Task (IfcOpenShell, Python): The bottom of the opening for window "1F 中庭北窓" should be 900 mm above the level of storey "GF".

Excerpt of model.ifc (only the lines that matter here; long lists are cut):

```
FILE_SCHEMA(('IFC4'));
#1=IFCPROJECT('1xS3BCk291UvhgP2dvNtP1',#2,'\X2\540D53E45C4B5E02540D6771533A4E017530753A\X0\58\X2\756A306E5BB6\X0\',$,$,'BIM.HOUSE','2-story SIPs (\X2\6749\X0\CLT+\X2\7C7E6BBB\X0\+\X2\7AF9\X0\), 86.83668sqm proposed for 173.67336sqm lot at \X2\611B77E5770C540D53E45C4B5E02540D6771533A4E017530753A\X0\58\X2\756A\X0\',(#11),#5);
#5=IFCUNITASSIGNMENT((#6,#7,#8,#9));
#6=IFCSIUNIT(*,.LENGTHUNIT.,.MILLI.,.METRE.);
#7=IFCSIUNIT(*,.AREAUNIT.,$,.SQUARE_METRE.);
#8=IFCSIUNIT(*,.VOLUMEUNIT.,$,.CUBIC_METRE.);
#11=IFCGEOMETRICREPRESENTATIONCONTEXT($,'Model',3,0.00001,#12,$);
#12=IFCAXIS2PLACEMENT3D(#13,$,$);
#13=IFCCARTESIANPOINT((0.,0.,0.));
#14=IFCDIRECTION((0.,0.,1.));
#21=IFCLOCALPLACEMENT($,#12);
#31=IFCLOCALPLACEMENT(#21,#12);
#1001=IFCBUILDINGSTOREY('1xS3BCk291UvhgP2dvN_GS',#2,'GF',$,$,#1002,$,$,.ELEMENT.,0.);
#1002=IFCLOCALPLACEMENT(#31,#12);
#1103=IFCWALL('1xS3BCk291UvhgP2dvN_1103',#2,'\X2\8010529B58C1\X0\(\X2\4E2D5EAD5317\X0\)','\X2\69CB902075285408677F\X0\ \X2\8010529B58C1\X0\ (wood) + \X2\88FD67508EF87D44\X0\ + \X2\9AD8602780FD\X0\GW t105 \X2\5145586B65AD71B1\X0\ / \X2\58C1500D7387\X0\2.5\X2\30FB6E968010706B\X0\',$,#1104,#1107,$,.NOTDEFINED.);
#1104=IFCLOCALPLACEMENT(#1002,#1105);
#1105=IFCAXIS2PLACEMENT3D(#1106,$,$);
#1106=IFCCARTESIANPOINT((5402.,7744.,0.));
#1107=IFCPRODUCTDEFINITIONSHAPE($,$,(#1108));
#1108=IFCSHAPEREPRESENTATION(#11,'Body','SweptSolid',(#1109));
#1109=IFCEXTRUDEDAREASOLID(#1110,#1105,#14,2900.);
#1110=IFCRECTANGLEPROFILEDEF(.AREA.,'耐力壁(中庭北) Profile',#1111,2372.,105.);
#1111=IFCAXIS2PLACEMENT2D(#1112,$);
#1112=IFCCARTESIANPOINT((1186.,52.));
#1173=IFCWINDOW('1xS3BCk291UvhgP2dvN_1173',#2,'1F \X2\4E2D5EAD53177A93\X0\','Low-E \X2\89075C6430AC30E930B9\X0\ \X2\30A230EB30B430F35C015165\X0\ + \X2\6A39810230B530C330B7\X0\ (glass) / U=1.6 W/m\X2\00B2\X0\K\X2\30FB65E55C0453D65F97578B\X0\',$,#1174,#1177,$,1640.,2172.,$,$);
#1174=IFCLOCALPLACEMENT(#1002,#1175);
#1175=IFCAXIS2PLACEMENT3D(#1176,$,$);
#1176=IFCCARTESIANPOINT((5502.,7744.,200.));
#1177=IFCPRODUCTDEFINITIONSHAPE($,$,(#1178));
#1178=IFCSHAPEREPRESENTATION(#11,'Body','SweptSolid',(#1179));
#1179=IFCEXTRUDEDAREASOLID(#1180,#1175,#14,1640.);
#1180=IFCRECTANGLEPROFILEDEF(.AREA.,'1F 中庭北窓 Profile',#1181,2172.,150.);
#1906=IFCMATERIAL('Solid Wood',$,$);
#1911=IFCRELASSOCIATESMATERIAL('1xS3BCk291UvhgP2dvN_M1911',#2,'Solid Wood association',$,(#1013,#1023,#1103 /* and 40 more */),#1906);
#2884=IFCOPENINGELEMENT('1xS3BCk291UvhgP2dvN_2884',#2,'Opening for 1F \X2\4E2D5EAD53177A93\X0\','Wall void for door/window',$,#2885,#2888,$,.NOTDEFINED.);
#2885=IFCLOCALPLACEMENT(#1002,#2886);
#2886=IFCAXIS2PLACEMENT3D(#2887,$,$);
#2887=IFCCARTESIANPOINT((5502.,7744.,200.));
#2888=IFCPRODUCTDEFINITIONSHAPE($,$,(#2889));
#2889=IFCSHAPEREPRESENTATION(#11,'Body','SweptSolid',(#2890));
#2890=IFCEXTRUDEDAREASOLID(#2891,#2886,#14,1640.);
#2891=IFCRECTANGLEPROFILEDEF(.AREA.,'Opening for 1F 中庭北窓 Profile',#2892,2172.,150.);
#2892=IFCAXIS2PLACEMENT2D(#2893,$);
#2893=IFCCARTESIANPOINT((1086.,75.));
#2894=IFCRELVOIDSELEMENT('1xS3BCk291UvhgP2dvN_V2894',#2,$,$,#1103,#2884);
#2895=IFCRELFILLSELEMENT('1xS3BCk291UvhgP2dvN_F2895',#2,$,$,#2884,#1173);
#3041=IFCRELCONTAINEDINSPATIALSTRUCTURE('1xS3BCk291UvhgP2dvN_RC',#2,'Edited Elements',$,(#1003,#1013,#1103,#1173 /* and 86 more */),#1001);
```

```python
import numpy as np
import ifcopenshell
import ifcopenshell.api.geometry
import ifcopenshell.geom
import ifcopenshell.util.element
import ifcopenshell.util.placement
import ifcopenshell.util.shape
import ifcopenshell.util.unit

model = ifcopenshell.open("model.ifc")
unit_scale = ifcopenshell.util.unit.calculate_unit_scale(model)

window = model.by_guid("1xS3BCk291UvhgP2dvN_1173")
opening = window.FillsVoids[0].RelatingOpeningElement
storey = ifcopenshell.util.element.get_container(window, ifc_class="IfcBuildingStorey")
level = ifcopenshell.util.placement.get_local_placement(storey.ObjectPlacement)[2, 3]

# The opening's origin need not be at the sill, so measure its lowest point.
shape = ifcopenshell.geom.create_shape(ifcopenshell.geom.settings(), opening)
bottom = ifcopenshell.util.shape.get_shape_bottom_elevation(shape, shape.geometry) / unit_scale
dz = level + 900.0 - bottom

shift = np.array([0.0, 0.0, dz])
# The window is not placed relative to its opening, so move both.
for product in (opening, window):
    matrix = ifcopenshell.util.placement.get_local_placement(product.ObjectPlacement)
    matrix[:3, 3] += shift
    ifcopenshell.api.geometry.edit_object_placement(model, product=product, matrix=matrix, is_si=False)

print(f"moved by {dz * unit_scale:+.3f} m")

model.write("model_updated.ifc")
```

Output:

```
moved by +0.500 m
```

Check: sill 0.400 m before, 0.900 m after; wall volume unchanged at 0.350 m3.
